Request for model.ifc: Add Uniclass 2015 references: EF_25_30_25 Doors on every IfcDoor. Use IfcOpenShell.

First a look at what the model holds.

```python
import ifcopenshell

model = ifcopenshell.open("model.ifc")
print(model.schema)
print("classifications:", [c.Name for c in model.by_type("IfcClassification")])
for ifc_class in ("IfcDoor", "IfcRoof", "IfcStair", "IfcWall", "IfcWindow"):
    print(ifc_class, len(model.by_type(ifc_class)))
```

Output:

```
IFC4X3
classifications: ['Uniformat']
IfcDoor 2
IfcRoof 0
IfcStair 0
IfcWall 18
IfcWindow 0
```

```python
import ifcopenshell
import ifcopenshell.api.classification

model = ifcopenshell.open("model.ifc")

system = ifcopenshell.api.classification.add_classification(model, classification="Uniclass 2015")

codes = {
    "IfcDoor": ("EF_25_30_25", "Doors"),
}
for ifc_class, (code, name) in codes.items():
    products = model.by_type(ifc_class)
    ifcopenshell.api.classification.add_reference(
        model, products=products, classification=system, identification=code, name=name
    )
    print(code, len(products))

model.write("model_updated.ifc")
```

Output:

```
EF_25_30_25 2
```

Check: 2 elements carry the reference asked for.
